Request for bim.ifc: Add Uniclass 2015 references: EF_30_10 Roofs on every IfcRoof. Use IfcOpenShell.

First a look at what the model holds.

```python
import ifcopenshell

model = ifcopenshell.open("bim.ifc")
print(model.schema)
print("classifications:", [c.Name for c in model.by_type("IfcClassification")])
for ifc_class in ("IfcDoor", "IfcRoof", "IfcStair", "IfcWall", "IfcWindow"):
    print(ifc_class, len(model.by_type(ifc_class)))
```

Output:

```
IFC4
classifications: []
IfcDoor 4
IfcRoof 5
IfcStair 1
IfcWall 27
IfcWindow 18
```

```python
import ifcopenshell
import ifcopenshell.api.classification

model = ifcopenshell.open("bim.ifc")

system = ifcopenshell.api.classification.add_classification(model, classification="Uniclass 2015")

codes = {
    "IfcRoof": ("EF_30_10", "Roofs"),
}
for ifc_class, (code, name) in codes.items():
    products = model.by_type(ifc_class)
    ifcopenshell.api.classification.add_reference(
        model, products=products, classification=system, identification=code, name=name
    )
    print(code, len(products))

model.write("bim_v2.ifc")
```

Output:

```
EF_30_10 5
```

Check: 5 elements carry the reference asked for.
